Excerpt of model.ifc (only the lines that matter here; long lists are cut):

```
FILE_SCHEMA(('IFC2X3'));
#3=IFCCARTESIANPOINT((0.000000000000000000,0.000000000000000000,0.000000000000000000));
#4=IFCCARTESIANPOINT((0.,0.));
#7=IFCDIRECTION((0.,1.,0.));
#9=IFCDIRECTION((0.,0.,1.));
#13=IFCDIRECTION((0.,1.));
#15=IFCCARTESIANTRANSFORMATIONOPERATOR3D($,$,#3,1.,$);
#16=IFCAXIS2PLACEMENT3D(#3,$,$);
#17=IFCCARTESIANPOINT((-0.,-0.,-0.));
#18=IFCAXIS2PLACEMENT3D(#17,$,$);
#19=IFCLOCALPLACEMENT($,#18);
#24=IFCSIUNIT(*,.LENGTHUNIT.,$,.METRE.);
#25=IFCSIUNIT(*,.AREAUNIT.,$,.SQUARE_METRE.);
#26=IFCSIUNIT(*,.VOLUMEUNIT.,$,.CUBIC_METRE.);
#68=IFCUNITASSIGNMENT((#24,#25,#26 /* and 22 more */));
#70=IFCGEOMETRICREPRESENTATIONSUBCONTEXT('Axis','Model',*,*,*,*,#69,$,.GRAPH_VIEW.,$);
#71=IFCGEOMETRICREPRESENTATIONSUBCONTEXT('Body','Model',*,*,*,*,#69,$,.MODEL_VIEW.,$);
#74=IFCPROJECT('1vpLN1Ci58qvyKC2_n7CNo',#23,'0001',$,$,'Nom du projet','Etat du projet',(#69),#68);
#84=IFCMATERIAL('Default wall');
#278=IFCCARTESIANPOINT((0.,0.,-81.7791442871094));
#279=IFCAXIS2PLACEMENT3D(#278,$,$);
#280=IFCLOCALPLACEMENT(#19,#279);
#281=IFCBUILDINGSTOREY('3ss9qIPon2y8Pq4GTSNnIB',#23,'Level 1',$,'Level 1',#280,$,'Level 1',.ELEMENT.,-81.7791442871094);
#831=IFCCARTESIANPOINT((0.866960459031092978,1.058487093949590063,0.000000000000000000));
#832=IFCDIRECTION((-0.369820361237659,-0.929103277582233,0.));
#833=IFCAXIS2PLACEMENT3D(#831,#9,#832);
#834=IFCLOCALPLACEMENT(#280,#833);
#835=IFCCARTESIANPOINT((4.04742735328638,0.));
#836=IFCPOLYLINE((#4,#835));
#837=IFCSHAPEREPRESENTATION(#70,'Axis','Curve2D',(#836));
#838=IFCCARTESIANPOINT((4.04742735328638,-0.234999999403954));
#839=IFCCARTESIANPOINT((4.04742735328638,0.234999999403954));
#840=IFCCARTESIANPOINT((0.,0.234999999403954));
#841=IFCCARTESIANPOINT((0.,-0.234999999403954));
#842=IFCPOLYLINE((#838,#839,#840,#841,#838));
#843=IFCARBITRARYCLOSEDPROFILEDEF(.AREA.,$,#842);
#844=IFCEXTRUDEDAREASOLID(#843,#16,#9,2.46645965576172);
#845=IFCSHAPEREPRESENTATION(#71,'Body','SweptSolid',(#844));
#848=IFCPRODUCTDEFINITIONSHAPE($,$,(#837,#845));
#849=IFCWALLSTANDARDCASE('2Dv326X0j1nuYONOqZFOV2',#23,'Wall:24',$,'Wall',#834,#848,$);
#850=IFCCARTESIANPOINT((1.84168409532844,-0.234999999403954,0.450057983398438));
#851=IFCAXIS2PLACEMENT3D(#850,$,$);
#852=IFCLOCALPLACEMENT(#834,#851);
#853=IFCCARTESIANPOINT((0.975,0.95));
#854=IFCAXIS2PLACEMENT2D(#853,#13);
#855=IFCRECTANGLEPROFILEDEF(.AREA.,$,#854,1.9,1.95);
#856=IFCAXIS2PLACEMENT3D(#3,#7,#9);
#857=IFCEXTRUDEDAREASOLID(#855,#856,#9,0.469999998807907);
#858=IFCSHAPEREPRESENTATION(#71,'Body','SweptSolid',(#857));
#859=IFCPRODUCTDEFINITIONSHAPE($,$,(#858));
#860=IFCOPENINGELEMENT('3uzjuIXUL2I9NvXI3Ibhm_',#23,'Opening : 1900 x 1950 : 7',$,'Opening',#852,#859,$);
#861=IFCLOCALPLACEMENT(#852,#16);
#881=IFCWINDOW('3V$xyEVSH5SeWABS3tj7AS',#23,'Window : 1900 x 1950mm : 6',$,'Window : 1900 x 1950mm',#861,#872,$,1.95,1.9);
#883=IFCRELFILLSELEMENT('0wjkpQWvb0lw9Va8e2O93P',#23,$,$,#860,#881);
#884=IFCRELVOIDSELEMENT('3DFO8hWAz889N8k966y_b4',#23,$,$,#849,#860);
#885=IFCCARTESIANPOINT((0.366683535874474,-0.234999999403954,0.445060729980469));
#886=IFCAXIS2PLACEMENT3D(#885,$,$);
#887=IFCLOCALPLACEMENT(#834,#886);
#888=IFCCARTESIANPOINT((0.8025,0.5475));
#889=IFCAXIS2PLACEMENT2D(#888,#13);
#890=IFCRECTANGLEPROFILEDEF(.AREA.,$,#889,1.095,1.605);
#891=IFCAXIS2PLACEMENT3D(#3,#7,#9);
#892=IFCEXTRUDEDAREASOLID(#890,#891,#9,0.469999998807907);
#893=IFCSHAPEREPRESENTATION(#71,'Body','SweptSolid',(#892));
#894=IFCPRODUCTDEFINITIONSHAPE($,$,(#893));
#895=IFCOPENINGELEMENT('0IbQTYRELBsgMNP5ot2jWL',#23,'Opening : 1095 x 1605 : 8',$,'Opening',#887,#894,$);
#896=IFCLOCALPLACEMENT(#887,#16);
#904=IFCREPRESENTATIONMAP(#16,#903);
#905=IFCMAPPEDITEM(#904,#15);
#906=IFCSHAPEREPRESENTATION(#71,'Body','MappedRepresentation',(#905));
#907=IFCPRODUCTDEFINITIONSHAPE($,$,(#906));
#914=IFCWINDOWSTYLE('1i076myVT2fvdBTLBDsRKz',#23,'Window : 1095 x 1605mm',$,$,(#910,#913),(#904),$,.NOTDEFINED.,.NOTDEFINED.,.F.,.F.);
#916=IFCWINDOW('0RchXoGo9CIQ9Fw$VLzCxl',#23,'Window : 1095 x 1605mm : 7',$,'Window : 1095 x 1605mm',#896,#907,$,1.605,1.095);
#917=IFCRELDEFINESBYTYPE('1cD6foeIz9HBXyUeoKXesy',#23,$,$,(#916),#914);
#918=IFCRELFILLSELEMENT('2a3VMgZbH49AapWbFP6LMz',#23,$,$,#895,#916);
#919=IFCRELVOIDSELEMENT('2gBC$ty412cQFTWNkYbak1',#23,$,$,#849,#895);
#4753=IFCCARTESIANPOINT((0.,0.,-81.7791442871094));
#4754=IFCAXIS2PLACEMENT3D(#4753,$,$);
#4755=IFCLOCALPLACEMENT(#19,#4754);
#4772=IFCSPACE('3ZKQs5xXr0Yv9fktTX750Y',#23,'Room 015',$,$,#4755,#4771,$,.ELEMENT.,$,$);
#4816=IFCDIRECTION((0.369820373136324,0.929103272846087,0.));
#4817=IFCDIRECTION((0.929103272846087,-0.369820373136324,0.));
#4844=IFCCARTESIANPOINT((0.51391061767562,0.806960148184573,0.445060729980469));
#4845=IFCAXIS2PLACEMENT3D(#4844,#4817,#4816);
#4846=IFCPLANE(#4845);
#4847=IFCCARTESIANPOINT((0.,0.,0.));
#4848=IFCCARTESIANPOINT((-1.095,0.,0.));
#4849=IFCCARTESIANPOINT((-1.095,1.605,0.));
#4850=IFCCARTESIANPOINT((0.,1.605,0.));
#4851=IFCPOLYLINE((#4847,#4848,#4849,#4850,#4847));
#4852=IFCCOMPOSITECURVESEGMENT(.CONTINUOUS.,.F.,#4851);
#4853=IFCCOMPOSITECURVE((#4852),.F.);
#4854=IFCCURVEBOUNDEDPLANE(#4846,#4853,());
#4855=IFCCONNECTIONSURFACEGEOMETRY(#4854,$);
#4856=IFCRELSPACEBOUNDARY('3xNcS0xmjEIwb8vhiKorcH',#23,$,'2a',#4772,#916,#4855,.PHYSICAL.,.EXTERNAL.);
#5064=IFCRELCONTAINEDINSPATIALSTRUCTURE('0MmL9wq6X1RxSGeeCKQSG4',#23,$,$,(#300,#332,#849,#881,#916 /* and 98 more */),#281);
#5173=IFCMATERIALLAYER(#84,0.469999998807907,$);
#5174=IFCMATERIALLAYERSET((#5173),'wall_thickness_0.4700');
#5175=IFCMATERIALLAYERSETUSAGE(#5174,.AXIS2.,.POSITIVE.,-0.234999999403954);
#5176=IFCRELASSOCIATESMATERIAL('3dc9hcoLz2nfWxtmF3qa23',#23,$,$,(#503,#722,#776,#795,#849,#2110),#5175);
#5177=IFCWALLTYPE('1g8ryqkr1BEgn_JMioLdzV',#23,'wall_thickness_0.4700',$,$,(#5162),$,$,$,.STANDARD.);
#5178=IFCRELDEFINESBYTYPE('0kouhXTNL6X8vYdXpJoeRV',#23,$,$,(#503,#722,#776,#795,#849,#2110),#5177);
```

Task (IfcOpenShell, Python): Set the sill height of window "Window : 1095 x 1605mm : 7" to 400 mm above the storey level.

```python
import numpy as np
import ifcopenshell
import ifcopenshell.api.geometry
import ifcopenshell.geom
import ifcopenshell.util.element
import ifcopenshell.util.placement
import ifcopenshell.util.shape
import ifcopenshell.util.unit

model = ifcopenshell.open("model.ifc")
unit_scale = ifcopenshell.util.unit.calculate_unit_scale(model)

window = model.by_id(916)
opening = window.FillsVoids[0].RelatingOpeningElement
storey = ifcopenshell.util.element.get_container(window, ifc_class="IfcBuildingStorey")
level = ifcopenshell.util.placement.get_local_placement(storey.ObjectPlacement)[2, 3]

# The opening's origin need not be at the sill, so measure its lowest point.
shape = ifcopenshell.geom.create_shape(ifcopenshell.geom.settings(), opening)
bottom = ifcopenshell.util.shape.get_shape_bottom_elevation(shape, shape.geometry) / unit_scale
dz = level + 0.4 - bottom

shift = np.array([0.0, 0.0, dz])
# The window is placed relative to its opening, so it follows when the opening moves.
matrix = ifcopenshell.util.placement.get_local_placement(opening.ObjectPlacement)
matrix[:3, 3] += shift
ifcopenshell.api.geometry.edit_object_placement(
    model, product=opening, matrix=matrix, is_si=False, should_transform_children=True
)

# Space boundary surfaces are stored in each space's coordinates; move them too.
for rel in window.ProvidesBoundaries:
    if not rel.ConnectionGeometry:
        continue
    surface = rel.ConnectionGeometry.SurfaceOnRelatingElement.BasisSurface
    space_matrix = ifcopenshell.util.placement.get_local_placement(rel.RelatingSpace.ObjectPlacement)
    point = np.array(surface.Position.Location.Coordinates) + space_matrix[:3, :3].T @ shift
    surface.Position = model.createIfcAxis2Placement3D(
        model.createIfcCartesianPoint(point.tolist()), surface.Position.Axis, surface.Position.RefDirection
    )

print(f"moved by {dz * unit_scale:+.3f} m")

model.write("model_rev.ifc")
```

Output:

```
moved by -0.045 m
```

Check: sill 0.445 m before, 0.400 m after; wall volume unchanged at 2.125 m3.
